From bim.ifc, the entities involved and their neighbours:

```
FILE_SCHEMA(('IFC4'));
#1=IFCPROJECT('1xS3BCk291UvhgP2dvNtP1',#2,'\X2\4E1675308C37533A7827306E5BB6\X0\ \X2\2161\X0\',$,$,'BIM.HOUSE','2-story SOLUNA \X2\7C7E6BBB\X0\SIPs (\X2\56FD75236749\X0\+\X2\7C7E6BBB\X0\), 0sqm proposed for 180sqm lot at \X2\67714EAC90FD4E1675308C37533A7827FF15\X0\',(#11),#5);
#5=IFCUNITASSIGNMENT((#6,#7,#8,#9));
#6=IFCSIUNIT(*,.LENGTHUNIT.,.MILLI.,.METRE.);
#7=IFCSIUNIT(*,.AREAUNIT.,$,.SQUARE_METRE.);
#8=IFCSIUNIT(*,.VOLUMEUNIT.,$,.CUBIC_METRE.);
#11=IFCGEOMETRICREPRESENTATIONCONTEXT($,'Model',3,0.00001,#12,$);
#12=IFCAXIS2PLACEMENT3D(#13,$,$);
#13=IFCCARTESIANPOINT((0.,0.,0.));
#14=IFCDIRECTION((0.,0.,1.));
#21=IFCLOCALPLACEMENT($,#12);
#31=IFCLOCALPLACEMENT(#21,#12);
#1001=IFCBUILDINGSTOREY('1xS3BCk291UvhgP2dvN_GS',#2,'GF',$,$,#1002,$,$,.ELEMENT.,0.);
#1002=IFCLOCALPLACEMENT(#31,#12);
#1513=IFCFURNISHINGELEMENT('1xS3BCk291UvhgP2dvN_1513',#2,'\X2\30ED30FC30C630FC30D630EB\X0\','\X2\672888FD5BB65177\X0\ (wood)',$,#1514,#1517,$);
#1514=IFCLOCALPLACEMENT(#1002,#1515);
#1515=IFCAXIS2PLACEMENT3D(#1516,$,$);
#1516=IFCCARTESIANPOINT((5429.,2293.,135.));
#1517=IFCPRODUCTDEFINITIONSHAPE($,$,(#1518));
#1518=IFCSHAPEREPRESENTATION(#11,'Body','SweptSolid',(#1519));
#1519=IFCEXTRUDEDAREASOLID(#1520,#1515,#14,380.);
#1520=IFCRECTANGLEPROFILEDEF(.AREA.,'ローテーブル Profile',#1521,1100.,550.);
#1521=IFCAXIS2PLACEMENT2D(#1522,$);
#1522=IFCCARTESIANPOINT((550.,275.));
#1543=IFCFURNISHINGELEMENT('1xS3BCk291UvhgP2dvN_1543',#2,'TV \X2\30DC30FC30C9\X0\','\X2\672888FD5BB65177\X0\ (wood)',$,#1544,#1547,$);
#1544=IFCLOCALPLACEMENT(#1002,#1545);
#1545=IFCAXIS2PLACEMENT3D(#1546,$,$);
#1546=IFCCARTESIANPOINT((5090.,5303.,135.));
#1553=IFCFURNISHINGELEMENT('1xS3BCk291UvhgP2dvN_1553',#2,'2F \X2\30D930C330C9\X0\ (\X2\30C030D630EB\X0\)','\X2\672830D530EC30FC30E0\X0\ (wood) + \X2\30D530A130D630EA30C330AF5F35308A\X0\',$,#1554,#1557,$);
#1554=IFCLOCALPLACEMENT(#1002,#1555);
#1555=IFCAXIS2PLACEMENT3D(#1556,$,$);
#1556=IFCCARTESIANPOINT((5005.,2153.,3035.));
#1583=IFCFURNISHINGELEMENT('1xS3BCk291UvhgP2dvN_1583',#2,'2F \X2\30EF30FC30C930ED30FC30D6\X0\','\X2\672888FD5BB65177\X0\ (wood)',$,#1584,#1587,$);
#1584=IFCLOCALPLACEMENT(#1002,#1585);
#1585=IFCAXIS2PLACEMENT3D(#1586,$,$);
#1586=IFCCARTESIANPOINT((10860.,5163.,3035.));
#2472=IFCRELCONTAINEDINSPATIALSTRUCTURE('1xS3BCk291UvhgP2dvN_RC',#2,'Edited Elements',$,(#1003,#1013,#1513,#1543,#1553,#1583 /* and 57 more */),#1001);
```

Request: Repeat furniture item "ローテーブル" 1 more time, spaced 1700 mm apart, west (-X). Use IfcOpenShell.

```python
import numpy as np
import ifcopenshell
import ifcopenshell.api.geometry
import ifcopenshell.api.root
import ifcopenshell.util.element
import ifcopenshell.util.placement
import ifcopenshell.util.unit

model = ifcopenshell.open("bim.ifc")
unit_scale = ifcopenshell.util.unit.calculate_unit_scale(model)


def reuse_history(source, copy):
    """copy_class also copies each property set's owner history, people and application; keep the originals."""
    for rel in copy.IsDefinedBy:
        if rel.is_a("IfcRelDefinesByProperties") and (history := rel.RelatingPropertyDefinition.OwnerHistory):
            rel.RelatingPropertyDefinition.OwnerHistory = source.OwnerHistory
            ifcopenshell.util.element.remove_deep2(model, history)


source = model.by_guid("1xS3BCk291UvhgP2dvN_1513")
base = ifcopenshell.util.placement.get_local_placement(source.ObjectPlacement)
step = np.array([-1.0, 0.0, 0.0]) * 1.7 / unit_scale

for i in range(1, 2):
    copy = ifcopenshell.api.root.copy_class(model, product=source)
    copy.Representation = ifcopenshell.util.element.copy_deep(
        model, source.Representation, exclude=["IfcGeometricRepresentationContext", "IfcRepresentationMap"]
    )
    reuse_history(source, copy)
    matrix = base.copy()
    matrix[:3, 3] += i * step
    print("added at", matrix[:3, 3].round(3) + 0.0)
    ifcopenshell.api.geometry.edit_object_placement(model, product=copy, matrix=matrix, is_si=False)

model.write("bim-out.ifc")
```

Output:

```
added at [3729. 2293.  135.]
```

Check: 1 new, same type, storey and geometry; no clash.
